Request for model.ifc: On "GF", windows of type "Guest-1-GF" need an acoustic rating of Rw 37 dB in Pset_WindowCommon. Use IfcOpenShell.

First a look at what the model holds.

```python
import ifcopenshell
import ifcopenshell.util.element

model = ifcopenshell.open("model.ifc")
print(model.schema)
storey = next(s for s in model.by_type("IfcBuildingStorey") if s.Name == "GF")
windows = [e for e in ifcopenshell.util.element.get_decomposition(storey) if e.is_a("IfcWindow")]
seen = {}
for e in windows:
    element_type = ifcopenshell.util.element.get_type(e)
    key = (element_type.Name if element_type != e and element_type else None, ifcopenshell.util.element.get_pset(e, "Pset_WindowCommon", "AcousticRating"))
    seen[key] = seen.get(key, 0) + 1
for (name, value), count in sorted(seen.items(), key=str):
    print(count, "x", name, "|", value)
```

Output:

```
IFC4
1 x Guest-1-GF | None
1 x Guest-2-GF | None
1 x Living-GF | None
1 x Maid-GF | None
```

```python
import ifcopenshell
import ifcopenshell.api.pset
import ifcopenshell.util.element

model = ifcopenshell.open("model.ifc")

storey = next(s for s in model.by_type("IfcBuildingStorey") if s.Name == "GF")
windows = [e for e in ifcopenshell.util.element.get_decomposition(storey) if e.is_a("IfcWindow")]

count = 0
for e in windows:
    element_type = ifcopenshell.util.element.get_type(e)
    if element_type in (None, e) or element_type.Name != "Guest-1-GF":
        continue
    # add_pset returns the element's existing set when there is one.
    pset = ifcopenshell.api.pset.add_pset(model, product=e, name="Pset_WindowCommon")
    ifcopenshell.api.pset.edit_pset(model, pset=pset, properties={"AcousticRating": "Rw 37 dB"})
    count += 1

print(count, "windows updated")

model.write("model-out.ifc")
```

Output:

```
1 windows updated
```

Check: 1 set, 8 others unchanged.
